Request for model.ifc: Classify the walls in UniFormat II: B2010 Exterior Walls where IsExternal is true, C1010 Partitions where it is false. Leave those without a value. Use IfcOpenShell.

First a look at what the model holds.

```python
import ifcopenshell
import ifcopenshell.util.element

model = ifcopenshell.open("model.ifc")
print(model.schema)
print("classifications:", [c.Name for c in model.by_type("IfcClassification")])
values = [ifcopenshell.util.element.get_pset(e, "Pset_WallCommon", "IsExternal") for e in model.by_type("IfcWall")]
for value in (True, False, None):
    print("IsExternal", value, values.count(value))
```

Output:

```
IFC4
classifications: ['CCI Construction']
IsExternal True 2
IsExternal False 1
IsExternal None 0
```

```python
import ifcopenshell
import ifcopenshell.api.classification
import ifcopenshell.util.element

model = ifcopenshell.open("model.ifc")

system = ifcopenshell.api.classification.add_classification(model, classification="UniFormat II")

walls = model.by_type("IfcWall")
external = {e: ifcopenshell.util.element.get_pset(e, "Pset_WallCommon", "IsExternal") for e in walls}
for flag, code, name in ((True, "B2010", "Exterior Walls"), (False, "C1010", "Partitions")):
    products = [e for e in walls if external[e] is flag]
    ifcopenshell.api.classification.add_reference(
        model, products=products, classification=system, identification=code, name=name
    )
    print(code, len(products))

model.write("model-out.ifc")
```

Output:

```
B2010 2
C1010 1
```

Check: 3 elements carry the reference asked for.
